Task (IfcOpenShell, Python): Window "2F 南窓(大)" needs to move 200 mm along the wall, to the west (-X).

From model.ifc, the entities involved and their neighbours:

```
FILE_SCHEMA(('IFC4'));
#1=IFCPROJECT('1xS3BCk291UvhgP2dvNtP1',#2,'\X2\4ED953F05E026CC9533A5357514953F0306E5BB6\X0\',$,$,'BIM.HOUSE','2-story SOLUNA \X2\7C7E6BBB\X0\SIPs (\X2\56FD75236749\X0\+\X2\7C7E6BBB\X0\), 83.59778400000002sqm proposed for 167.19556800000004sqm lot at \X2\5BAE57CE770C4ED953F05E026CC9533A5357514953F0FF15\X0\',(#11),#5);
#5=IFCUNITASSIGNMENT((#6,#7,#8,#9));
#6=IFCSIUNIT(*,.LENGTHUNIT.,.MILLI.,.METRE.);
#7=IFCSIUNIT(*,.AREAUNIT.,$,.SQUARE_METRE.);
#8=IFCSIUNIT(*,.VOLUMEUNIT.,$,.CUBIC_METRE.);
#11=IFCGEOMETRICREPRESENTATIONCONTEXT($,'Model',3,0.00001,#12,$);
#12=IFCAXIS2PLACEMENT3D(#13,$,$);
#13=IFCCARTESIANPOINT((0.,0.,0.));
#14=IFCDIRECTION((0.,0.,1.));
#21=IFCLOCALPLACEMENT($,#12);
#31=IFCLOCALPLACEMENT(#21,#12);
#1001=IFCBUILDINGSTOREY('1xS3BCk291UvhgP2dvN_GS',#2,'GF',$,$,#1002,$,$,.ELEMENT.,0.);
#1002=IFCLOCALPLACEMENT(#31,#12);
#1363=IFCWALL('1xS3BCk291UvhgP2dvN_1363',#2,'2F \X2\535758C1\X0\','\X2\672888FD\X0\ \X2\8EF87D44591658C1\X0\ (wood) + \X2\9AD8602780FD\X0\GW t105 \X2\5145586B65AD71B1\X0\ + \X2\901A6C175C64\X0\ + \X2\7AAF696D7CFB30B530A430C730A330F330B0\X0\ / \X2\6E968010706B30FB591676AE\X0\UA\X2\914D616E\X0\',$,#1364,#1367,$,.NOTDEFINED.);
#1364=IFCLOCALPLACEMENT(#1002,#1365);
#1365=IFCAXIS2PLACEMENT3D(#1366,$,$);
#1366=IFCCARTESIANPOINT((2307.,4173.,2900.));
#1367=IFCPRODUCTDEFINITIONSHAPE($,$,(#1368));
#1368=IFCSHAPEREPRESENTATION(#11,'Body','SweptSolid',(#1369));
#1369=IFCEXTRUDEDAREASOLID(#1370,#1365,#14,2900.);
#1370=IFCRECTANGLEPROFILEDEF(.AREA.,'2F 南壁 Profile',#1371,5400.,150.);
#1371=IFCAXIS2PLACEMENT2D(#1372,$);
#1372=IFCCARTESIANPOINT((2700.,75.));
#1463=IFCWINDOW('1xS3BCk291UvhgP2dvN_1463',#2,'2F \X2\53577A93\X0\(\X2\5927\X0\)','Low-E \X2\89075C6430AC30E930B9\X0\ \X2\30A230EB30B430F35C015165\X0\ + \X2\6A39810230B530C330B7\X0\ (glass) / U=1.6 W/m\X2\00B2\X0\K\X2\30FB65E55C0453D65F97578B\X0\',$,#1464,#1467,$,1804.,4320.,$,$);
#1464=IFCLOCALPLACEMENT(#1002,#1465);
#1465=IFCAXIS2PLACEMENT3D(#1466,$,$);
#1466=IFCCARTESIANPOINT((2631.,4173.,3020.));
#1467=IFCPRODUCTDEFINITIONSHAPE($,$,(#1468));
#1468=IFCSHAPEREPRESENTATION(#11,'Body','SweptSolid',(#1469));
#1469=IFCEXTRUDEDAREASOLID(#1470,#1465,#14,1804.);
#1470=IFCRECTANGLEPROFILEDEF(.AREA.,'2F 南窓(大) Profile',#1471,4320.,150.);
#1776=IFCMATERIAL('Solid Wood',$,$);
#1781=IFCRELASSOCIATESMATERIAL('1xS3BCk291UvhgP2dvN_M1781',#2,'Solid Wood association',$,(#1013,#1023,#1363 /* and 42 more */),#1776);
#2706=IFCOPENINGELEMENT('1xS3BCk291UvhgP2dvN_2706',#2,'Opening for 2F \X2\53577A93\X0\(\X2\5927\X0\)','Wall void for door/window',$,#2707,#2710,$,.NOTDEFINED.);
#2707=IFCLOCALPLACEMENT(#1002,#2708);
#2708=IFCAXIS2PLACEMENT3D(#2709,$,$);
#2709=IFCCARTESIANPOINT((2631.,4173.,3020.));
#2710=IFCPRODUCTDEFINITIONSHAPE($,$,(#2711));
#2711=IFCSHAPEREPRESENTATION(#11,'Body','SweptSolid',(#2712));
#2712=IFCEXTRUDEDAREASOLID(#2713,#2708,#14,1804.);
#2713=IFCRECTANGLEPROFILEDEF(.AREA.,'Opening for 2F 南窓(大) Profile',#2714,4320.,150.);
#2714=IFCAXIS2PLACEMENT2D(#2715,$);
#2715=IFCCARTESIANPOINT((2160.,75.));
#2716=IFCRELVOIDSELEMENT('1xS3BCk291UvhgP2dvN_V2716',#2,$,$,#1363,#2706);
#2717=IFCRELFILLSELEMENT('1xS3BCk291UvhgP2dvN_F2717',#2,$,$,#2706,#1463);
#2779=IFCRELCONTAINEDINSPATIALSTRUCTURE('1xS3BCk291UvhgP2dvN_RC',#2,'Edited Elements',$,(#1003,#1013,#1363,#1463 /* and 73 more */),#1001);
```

```python
import ifcopenshell
import ifcopenshell.api.geometry
import ifcopenshell.util.placement

model = ifcopenshell.open("model.ifc")

window = model.by_id(1463)
opening = window.FillsVoids[0].RelatingOpeningElement
wall = opening.VoidsElements[0].RelatingBuildingElement

wall_matrix = ifcopenshell.util.placement.get_local_placement(wall.ObjectPlacement)
shift = wall_matrix[:3, 0] * -200.0
before = ifcopenshell.util.placement.get_local_placement(window.ObjectPlacement)[:3, 3].copy()

# The window is not placed relative to its opening, so move both.
for product in (opening, window):
    matrix = ifcopenshell.util.placement.get_local_placement(product.ObjectPlacement)
    matrix[:3, 3] += shift
    ifcopenshell.api.geometry.edit_object_placement(model, product=product, matrix=matrix, is_si=False)

after = ifcopenshell.util.placement.get_local_placement(window.ObjectPlacement)[:3, 3]
print("window moved by", (after - before).round(3) + 0.0)

model.write("model_v2.ifc")
```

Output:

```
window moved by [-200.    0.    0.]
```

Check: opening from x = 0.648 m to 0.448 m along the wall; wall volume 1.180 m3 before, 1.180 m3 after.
